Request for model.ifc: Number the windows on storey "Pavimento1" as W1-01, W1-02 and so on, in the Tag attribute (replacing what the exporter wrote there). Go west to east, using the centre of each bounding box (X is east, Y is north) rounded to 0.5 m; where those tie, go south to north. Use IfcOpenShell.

First a look at what the model holds.

```python
import ifcopenshell
import ifcopenshell.util.element
import ifcopenshell.util.placement

model = ifcopenshell.open("model.ifc")
print(model.schema)
storey = next(s for s in model.by_type("IfcBuildingStorey") if s.Name == "Pavimento1")
windows = [e for e in ifcopenshell.util.element.get_decomposition(storey) if e.is_a("IfcWindow")]
for e in sorted(windows, key=lambda e: e.id()):
    origin = ifcopenshell.util.placement.get_local_placement(e.ObjectPlacement)[:3, 3]
    print(e.id(), e.Tag, e.Name, origin.round(2) + 0.0, sep=" | ")
```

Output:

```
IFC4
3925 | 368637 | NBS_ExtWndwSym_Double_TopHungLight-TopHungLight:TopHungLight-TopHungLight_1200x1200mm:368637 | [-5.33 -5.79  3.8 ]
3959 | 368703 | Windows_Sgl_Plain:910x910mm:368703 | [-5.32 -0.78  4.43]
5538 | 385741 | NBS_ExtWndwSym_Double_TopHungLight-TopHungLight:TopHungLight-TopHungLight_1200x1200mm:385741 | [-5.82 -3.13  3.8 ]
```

```python
import ifcopenshell
import ifcopenshell.geom
import ifcopenshell.util.element
import ifcopenshell.util.shape

model = ifcopenshell.open("model.ifc")
settings = ifcopenshell.geom.settings()
settings.set("use-world-coords", True)


def centre(element):
    shape = ifcopenshell.geom.create_shape(settings, element)
    return ifcopenshell.util.shape.get_bbox_centroid(shape.geometry)


storey = next(s for s in model.by_type("IfcBuildingStorey") if s.Name == "Pavimento1")
windows = [e for e in ifcopenshell.util.element.get_decomposition(storey) if e.is_a("IfcWindow")]

# Insertion points can sit at a corner or the storey origin, so sort by the geometry (in metres).
centres = {e: centre(e) for e in windows}
windows.sort(key=lambda e: (round(centres[e][0] / 0.5), centres[e][1]))

for i, e in enumerate(windows, start=1):
    number = f"W1-{i:02d}"
    e.Tag = number
    print(e.id(), number)

model.write("model_rev.ifc")
```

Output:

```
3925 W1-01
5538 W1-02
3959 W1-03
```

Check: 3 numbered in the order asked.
